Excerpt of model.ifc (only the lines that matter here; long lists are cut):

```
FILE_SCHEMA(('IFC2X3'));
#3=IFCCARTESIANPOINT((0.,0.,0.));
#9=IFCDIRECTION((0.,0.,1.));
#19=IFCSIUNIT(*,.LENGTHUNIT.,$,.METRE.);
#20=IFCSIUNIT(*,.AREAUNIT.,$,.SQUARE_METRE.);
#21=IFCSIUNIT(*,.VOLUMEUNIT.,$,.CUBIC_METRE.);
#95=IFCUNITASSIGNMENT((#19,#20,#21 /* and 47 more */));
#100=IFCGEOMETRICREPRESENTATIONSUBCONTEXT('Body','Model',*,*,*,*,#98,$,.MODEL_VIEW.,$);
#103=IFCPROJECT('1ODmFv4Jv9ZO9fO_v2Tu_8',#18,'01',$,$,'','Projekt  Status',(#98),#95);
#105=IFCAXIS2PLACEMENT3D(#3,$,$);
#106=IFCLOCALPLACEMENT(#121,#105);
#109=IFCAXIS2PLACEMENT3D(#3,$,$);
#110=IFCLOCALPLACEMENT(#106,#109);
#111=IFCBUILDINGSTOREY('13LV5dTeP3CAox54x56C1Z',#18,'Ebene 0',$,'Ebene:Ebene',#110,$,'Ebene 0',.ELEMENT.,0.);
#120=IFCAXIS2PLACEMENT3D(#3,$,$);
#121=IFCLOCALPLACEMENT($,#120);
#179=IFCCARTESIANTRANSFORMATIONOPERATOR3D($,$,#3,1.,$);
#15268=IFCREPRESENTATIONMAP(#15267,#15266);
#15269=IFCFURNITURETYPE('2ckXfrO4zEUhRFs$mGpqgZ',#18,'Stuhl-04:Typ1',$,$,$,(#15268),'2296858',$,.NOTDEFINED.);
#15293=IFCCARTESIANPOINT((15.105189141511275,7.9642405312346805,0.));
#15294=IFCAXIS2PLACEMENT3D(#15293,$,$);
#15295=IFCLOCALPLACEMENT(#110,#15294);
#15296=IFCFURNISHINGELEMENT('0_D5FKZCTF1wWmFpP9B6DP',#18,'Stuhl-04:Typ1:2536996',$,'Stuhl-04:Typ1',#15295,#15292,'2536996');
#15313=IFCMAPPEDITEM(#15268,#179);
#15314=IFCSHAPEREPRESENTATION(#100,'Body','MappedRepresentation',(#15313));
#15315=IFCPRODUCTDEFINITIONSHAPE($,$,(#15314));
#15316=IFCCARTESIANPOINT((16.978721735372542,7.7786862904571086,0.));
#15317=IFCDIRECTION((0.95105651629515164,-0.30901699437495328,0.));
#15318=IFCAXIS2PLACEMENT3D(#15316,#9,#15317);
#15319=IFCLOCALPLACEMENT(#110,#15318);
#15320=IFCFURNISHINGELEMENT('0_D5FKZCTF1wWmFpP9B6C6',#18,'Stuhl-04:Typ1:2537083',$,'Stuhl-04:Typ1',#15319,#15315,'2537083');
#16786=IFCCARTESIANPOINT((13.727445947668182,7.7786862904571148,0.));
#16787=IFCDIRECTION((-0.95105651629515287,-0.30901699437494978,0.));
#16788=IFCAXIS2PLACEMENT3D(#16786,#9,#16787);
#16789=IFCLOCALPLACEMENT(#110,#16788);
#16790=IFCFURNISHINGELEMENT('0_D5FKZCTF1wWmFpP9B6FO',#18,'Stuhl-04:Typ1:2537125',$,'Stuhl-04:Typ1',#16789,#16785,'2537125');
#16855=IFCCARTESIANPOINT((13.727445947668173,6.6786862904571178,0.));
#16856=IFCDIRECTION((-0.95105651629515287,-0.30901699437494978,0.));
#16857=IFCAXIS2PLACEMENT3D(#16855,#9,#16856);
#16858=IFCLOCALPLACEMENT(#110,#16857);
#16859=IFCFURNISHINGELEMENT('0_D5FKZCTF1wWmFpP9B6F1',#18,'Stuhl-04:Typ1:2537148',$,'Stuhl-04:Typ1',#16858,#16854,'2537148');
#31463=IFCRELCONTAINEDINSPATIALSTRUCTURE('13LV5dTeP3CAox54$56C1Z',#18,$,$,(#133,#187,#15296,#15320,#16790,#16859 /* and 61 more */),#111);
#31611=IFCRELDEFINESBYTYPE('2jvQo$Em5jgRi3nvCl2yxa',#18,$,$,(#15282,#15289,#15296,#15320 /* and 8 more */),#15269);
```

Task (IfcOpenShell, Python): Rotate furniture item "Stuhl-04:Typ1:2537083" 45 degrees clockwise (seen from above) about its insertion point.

```python
import ifcopenshell
import ifcopenshell.api.geometry
import ifcopenshell.util.placement

model = ifcopenshell.open("model.ifc")

item = model.by_guid("0_D5FKZCTF1wWmFpP9B6C6")
matrix = ifcopenshell.util.placement.get_local_placement(item.ObjectPlacement)
matrix = matrix @ ifcopenshell.util.placement.rotation(-45, "Z")
ifcopenshell.api.geometry.edit_object_placement(model, product=item, matrix=matrix, is_si=False)

print(ifcopenshell.util.placement.get_local_placement(item.ObjectPlacement).round(3) + 0.0)

model.write("model_edited.ifc")
```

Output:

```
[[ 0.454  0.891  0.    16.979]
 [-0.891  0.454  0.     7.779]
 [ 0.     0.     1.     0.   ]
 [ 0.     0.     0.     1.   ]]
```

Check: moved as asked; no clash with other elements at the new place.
